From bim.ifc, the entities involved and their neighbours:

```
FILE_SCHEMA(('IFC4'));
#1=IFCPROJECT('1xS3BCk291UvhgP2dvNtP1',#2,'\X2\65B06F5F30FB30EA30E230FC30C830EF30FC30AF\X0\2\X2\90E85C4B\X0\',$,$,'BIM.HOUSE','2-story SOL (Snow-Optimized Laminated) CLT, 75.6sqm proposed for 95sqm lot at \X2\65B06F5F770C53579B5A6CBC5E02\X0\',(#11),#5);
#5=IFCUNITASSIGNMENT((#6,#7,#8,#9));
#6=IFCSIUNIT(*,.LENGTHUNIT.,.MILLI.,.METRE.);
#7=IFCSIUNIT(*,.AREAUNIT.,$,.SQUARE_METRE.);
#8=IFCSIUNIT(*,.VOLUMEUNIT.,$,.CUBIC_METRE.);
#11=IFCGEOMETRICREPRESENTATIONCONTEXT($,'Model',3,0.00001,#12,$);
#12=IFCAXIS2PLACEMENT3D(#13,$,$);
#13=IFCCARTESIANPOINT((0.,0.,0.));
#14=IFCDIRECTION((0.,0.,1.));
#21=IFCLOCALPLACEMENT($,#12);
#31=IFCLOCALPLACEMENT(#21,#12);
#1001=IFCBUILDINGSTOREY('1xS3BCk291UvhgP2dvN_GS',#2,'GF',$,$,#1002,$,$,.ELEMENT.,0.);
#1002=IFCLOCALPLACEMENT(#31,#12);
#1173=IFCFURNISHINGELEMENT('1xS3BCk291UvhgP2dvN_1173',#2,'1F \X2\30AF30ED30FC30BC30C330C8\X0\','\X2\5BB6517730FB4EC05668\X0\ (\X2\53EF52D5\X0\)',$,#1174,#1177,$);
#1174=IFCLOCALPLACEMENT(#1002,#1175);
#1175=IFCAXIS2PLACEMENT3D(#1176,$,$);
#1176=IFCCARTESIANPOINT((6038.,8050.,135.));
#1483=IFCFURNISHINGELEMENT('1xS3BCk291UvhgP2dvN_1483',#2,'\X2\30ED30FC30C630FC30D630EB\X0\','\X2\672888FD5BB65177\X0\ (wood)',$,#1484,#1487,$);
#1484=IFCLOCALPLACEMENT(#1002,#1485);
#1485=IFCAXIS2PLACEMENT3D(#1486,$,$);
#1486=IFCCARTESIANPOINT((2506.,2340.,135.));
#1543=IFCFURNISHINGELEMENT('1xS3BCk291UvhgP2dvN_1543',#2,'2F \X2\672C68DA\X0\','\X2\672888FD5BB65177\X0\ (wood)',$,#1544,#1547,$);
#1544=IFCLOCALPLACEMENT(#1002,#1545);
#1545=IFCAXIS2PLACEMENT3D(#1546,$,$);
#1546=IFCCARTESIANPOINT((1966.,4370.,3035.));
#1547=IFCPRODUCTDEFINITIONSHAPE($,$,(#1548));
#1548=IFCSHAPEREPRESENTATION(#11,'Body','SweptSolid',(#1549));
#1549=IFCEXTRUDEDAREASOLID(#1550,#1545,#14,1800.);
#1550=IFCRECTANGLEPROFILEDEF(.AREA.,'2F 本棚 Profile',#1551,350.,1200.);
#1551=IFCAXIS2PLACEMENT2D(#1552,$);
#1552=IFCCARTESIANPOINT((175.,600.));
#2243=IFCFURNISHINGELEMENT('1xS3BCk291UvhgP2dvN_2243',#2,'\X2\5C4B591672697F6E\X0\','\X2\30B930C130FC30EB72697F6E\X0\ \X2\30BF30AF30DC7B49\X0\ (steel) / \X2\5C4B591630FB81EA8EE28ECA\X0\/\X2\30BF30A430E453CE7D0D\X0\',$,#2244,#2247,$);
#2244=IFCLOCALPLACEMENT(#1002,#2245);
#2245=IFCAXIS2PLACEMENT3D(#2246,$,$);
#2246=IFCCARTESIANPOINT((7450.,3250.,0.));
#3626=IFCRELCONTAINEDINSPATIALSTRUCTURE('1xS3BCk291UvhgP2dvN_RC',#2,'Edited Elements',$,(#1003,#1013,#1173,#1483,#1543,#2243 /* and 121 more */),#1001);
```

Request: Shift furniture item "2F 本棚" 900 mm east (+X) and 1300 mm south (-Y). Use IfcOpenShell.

```python
import ifcopenshell
import ifcopenshell.api.geometry
import ifcopenshell.util.placement
import ifcopenshell.util.unit

model = ifcopenshell.open("bim.ifc")
unit_scale = ifcopenshell.util.unit.calculate_unit_scale(model)

item = model.by_id(1543)
matrix = ifcopenshell.util.placement.get_local_placement(item.ObjectPlacement)
matrix[0, 3] += 0.9 / unit_scale
matrix[1, 3] -= 1.3 / unit_scale
ifcopenshell.api.geometry.edit_object_placement(model, product=item, matrix=matrix, is_si=False)

print(ifcopenshell.util.placement.get_local_placement(item.ObjectPlacement).round(3) + 0.0)

model.write("bim_updated.ifc")
```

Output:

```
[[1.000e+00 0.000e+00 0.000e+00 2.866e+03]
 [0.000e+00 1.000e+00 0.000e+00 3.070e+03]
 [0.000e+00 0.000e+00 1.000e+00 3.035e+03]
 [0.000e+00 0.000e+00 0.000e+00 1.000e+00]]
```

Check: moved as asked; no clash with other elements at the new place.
